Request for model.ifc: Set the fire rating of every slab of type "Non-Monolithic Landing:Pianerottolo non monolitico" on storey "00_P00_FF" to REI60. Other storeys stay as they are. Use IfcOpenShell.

First a look at what the model holds.

```python
import ifcopenshell
import ifcopenshell.util.element

model = ifcopenshell.open("model.ifc")
print(model.schema)
storey = next(s for s in model.by_type("IfcBuildingStorey") if s.Name == "00_P00_FF")
slabs = [e for e in ifcopenshell.util.element.get_decomposition(storey) if e.is_a("IfcSlab")]
seen = {}
for e in slabs:
    element_type = ifcopenshell.util.element.get_type(e)
    key = (element_type.Name if element_type != e and element_type else None, ifcopenshell.util.element.get_pset(e, "Pset_SlabCommon", "FireRating"))
    seen[key] = seen.get(key, 0) + 1
for (name, value), count in sorted(seen.items(), key=str):
    print(count, "x", name, "|", value)
```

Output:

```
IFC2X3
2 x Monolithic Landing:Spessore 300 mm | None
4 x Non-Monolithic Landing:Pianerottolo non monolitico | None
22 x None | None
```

```python
import ifcopenshell
import ifcopenshell.api.pset
import ifcopenshell.util.element

model = ifcopenshell.open("model.ifc")

storey = next(s for s in model.by_type("IfcBuildingStorey") if s.Name == "00_P00_FF")
slabs = [e for e in ifcopenshell.util.element.get_decomposition(storey) if e.is_a("IfcSlab")]

count = 0
for e in slabs:
    element_type = ifcopenshell.util.element.get_type(e)
    if element_type in (None, e) or element_type.Name != "Non-Monolithic Landing:Pianerottolo non monolitico":
        continue
    # add_pset returns the element's existing set when there is one.
    pset = ifcopenshell.api.pset.add_pset(model, product=e, name="Pset_SlabCommon")
    ifcopenshell.api.pset.edit_pset(model, pset=pset, properties={"FireRating": "REI60"})
    count += 1

print(count, "slabs updated")

model.write("model_updated.ifc")
```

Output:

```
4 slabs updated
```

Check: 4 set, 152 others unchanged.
